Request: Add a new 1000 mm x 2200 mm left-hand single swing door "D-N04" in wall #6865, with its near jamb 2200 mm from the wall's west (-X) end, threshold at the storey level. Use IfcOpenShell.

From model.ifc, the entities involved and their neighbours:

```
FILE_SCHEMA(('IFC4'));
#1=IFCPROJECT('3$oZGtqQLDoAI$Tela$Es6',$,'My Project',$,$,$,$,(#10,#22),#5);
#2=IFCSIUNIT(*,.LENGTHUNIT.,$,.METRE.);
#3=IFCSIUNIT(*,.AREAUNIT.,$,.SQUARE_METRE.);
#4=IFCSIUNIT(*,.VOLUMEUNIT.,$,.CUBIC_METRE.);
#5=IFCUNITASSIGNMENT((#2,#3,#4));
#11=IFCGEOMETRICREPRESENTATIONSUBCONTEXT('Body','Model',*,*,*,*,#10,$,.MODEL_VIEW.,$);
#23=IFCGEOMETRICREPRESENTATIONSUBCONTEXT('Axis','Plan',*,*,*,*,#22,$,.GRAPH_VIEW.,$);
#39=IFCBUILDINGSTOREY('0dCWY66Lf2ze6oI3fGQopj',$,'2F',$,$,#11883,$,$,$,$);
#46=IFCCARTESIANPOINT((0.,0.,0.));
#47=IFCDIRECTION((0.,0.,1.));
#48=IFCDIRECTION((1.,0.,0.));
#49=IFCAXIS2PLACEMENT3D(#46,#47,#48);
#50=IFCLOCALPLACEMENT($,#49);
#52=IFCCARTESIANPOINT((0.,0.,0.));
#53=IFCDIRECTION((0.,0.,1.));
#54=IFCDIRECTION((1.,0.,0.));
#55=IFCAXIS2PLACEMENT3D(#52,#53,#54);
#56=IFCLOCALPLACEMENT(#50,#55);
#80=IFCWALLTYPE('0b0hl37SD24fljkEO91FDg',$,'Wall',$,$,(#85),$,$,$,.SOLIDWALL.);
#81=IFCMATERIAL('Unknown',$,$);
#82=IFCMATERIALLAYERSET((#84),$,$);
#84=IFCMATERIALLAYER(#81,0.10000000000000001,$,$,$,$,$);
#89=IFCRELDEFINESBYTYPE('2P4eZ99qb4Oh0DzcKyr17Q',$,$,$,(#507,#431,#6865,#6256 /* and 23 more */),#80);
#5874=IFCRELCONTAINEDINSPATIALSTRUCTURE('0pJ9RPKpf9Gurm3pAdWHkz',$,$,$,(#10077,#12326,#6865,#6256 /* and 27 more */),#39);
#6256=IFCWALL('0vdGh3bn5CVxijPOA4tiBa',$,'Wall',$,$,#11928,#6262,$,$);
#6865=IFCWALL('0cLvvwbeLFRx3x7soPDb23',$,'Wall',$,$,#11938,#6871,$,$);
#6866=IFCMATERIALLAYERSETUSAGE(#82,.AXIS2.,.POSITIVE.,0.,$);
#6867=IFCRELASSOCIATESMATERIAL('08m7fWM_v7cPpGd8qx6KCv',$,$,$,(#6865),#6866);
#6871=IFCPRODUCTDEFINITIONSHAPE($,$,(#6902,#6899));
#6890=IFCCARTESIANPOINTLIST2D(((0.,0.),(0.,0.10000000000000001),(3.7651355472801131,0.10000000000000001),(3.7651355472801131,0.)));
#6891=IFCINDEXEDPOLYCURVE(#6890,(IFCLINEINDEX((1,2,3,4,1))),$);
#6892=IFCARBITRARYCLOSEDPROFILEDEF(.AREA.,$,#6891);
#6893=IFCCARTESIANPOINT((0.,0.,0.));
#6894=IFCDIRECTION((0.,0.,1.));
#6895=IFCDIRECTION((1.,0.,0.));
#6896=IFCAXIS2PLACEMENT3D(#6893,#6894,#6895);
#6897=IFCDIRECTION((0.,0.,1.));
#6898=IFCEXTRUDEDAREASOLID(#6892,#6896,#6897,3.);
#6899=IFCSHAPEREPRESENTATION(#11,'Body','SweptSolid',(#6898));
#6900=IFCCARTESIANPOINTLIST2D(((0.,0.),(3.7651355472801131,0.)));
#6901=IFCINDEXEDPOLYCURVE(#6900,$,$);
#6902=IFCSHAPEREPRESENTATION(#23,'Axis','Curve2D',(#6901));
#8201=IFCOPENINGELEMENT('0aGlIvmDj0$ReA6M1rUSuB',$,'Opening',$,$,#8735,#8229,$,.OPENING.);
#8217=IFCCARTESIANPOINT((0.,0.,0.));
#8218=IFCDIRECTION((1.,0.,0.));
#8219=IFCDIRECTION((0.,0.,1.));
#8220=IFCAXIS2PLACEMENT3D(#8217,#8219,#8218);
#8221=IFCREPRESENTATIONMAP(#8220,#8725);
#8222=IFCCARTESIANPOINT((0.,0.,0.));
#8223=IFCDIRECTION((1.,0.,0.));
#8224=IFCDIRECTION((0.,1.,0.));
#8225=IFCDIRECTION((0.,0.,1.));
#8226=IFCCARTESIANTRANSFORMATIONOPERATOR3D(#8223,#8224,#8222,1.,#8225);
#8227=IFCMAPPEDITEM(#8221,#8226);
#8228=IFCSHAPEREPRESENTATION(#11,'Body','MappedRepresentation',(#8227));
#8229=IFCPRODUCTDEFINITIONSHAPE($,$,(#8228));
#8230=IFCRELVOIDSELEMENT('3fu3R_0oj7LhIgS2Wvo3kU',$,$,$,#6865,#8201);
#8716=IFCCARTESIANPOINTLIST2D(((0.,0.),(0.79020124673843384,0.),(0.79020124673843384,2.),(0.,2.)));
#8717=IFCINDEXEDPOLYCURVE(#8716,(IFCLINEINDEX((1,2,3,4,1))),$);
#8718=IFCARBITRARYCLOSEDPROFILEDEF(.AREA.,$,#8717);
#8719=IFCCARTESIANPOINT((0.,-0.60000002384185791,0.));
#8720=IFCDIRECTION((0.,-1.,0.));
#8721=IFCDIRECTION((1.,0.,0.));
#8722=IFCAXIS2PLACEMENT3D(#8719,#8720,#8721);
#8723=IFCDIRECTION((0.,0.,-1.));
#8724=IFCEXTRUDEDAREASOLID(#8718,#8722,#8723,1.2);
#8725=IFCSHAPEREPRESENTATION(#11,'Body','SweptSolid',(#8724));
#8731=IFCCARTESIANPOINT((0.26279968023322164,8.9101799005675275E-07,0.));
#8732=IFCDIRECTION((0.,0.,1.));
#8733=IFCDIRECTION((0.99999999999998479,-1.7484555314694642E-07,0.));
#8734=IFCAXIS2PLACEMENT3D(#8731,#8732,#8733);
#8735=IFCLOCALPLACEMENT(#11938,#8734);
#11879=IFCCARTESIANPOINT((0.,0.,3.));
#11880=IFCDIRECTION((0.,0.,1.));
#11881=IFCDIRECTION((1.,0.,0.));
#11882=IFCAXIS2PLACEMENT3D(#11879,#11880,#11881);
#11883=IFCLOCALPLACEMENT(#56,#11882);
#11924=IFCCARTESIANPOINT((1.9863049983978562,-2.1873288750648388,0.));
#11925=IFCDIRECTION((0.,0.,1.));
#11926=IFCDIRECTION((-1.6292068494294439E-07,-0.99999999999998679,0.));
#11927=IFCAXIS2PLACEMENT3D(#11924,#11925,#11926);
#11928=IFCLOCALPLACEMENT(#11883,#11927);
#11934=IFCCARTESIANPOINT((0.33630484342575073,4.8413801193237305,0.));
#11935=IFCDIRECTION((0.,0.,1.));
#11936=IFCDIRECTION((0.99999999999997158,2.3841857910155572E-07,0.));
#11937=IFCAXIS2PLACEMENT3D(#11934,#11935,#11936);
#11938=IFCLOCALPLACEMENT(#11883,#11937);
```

```python
import numpy as np
import ifcopenshell
import ifcopenshell.api.feature
import ifcopenshell.api.geometry
import ifcopenshell.api.root
import ifcopenshell.api.spatial
import ifcopenshell.geom
import ifcopenshell.util.element
import ifcopenshell.util.placement
import ifcopenshell.util.representation
import ifcopenshell.util.shape
import ifcopenshell.util.unit

model = ifcopenshell.open("model.ifc")
unit_scale = ifcopenshell.util.unit.calculate_unit_scale(model)
settings = ifcopenshell.geom.settings()


def volume(element):
    """Net volume in cubic metres, openings subtracted."""
    shape = ifcopenshell.geom.create_shape(settings, element)
    return ifcopenshell.util.shape.get_volume(shape.geometry)


wall = model.by_guid("0cLvvwbeLFRx3x7soPDb23")
storey = ifcopenshell.util.element.get_container(wall, ifc_class="IfcBuildingStorey")
context = ifcopenshell.util.representation.get_context(model, "Model", "Body", "MODEL_VIEW")
before = volume(wall)

width, height, from_end, sill = 1, 2.2, 2.2, 0.0  # metres

# The wall runs along its own X axis, and the end named is its -X end.
wall_shape = ifcopenshell.geom.create_shape(settings, wall)
x, y, z = ifcopenshell.util.shape.get_vertices(wall_shape.geometry).T
start = x.min() + from_end
face, thickness = float(y.min()), float(y.max() - y.min())
wall_matrix = ifcopenshell.util.placement.get_local_placement(wall.ObjectPlacement)
level = ifcopenshell.util.placement.get_local_placement(storey.ObjectPlacement)[2, 3]


def in_wall(x, y):
    """Placement at x, y metres in the wall's axes, at sill height."""
    matrix = wall_matrix.copy()
    matrix[:, 3] = wall_matrix @ np.array([x / unit_scale, y / unit_scale, 0.0, 1.0])
    matrix[2, 3] = level + sill / unit_scale
    return matrix


# Opening: a box that overshoots both wall faces by 50 mm.
opening = ifcopenshell.api.root.create_entity(model, ifc_class="IfcOpeningElement", predefined_type="OPENING")
box = ifcopenshell.api.geometry.add_wall_representation(
    model, context=context, length=width, height=height, thickness=thickness + 0.1
)
ifcopenshell.api.geometry.assign_representation(model, product=opening, representation=box)
ifcopenshell.api.geometry.edit_object_placement(model, product=opening, matrix=in_wall(start, face - 0.05), is_si=False)
ifcopenshell.api.feature.add_feature(model, feature=opening, element=wall)

door = ifcopenshell.api.root.create_entity(model, ifc_class="IfcDoor", name="D-N04", predefined_type="DOOR")
door.OverallWidth, door.OverallHeight = width / unit_scale, height / unit_scale
door.OperationType = "SINGLE_SWING_LEFT"
body = ifcopenshell.api.geometry.add_door_representation(
    model,
    context=context,
    overall_width=door.OverallWidth,
    overall_height=door.OverallHeight,
    operation_type="SINGLE_SWING_LEFT",
    lining_properties={"LiningDepth": thickness / unit_scale, "ThresholdDepth": thickness / unit_scale},
)
ifcopenshell.api.geometry.assign_representation(model, product=door, representation=body)
ifcopenshell.api.spatial.assign_container(model, products=[door], relating_structure=storey)
ifcopenshell.api.feature.add_filling(model, opening=opening, element=door)

# The lining spans the wall, so the door starts at the wall face.
ifcopenshell.api.geometry.edit_object_placement(model, product=door, matrix=in_wall(start, face), is_si=False)

after = volume(wall)

print(f"wall volume {before:.3f} -> {after:.3f} m3")

model.write("model_v2.ifc")
```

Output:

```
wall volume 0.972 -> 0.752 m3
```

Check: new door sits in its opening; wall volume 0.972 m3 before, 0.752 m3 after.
